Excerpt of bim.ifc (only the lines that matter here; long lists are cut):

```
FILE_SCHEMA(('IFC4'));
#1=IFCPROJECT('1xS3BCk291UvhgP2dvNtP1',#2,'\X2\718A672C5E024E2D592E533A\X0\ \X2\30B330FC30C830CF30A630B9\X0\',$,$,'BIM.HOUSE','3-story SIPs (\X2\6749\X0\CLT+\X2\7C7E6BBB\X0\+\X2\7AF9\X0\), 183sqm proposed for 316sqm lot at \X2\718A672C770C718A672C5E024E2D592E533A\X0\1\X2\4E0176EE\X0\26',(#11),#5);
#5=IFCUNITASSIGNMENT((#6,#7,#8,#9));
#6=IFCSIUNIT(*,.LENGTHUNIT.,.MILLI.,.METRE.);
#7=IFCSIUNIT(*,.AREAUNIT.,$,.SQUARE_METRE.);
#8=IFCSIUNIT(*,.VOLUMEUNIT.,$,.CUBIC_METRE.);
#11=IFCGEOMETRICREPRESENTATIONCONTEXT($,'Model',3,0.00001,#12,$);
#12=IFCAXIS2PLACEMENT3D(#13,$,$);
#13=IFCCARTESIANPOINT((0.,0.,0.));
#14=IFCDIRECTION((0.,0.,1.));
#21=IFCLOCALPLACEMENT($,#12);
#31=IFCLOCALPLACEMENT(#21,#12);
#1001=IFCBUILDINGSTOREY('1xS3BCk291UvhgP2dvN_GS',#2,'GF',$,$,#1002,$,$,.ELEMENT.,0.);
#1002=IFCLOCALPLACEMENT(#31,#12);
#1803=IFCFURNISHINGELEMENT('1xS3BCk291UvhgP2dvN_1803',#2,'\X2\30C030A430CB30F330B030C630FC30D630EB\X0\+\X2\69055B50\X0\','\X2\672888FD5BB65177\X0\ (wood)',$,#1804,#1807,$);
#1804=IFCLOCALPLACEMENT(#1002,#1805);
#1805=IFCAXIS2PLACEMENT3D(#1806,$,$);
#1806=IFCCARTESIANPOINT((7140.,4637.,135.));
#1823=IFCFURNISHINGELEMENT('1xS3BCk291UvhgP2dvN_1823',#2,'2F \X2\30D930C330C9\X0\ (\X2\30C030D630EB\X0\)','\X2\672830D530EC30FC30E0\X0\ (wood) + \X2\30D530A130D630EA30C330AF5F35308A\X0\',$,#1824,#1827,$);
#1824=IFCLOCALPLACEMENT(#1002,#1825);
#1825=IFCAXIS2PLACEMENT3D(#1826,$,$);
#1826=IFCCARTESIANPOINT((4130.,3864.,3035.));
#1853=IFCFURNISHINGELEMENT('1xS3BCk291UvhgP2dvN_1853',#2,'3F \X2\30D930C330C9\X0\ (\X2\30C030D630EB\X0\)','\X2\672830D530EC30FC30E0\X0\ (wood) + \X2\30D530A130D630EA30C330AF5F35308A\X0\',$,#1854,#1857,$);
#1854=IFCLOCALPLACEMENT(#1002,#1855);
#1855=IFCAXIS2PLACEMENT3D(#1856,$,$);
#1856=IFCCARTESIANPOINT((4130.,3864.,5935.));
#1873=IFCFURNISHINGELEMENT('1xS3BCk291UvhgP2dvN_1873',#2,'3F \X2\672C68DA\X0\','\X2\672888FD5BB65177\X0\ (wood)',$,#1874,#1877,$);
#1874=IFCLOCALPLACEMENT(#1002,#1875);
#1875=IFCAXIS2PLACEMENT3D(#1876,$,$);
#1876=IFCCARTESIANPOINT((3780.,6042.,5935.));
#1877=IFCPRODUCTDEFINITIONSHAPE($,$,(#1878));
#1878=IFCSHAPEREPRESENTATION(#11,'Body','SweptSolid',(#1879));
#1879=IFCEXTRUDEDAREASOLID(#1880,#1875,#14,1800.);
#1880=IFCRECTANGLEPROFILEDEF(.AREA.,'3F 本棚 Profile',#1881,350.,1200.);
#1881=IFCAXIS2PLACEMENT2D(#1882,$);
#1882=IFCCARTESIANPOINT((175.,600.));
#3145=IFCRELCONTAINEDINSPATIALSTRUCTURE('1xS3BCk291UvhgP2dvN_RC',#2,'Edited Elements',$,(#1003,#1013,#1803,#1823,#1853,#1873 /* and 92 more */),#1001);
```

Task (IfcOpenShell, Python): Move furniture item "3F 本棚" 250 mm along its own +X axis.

```python
import ifcopenshell
import ifcopenshell.api.geometry
import ifcopenshell.util.placement
import ifcopenshell.util.unit

model = ifcopenshell.open("bim.ifc")
unit_scale = ifcopenshell.util.unit.calculate_unit_scale(model)

item = model.by_guid("1xS3BCk291UvhgP2dvN_1873")
matrix = ifcopenshell.util.placement.get_local_placement(item.ObjectPlacement)
matrix[:3, 3] += matrix[:3, 0] * 0.25 / unit_scale
ifcopenshell.api.geometry.edit_object_placement(model, product=item, matrix=matrix, is_si=False)

print(ifcopenshell.util.placement.get_local_placement(item.ObjectPlacement).round(3) + 0.0)

model.write("bim_rev.ifc")
```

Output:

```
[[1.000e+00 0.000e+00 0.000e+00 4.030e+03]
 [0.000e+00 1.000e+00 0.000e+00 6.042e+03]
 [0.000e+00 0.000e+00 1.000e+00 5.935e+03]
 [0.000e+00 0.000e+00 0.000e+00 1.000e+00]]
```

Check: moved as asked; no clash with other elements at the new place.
